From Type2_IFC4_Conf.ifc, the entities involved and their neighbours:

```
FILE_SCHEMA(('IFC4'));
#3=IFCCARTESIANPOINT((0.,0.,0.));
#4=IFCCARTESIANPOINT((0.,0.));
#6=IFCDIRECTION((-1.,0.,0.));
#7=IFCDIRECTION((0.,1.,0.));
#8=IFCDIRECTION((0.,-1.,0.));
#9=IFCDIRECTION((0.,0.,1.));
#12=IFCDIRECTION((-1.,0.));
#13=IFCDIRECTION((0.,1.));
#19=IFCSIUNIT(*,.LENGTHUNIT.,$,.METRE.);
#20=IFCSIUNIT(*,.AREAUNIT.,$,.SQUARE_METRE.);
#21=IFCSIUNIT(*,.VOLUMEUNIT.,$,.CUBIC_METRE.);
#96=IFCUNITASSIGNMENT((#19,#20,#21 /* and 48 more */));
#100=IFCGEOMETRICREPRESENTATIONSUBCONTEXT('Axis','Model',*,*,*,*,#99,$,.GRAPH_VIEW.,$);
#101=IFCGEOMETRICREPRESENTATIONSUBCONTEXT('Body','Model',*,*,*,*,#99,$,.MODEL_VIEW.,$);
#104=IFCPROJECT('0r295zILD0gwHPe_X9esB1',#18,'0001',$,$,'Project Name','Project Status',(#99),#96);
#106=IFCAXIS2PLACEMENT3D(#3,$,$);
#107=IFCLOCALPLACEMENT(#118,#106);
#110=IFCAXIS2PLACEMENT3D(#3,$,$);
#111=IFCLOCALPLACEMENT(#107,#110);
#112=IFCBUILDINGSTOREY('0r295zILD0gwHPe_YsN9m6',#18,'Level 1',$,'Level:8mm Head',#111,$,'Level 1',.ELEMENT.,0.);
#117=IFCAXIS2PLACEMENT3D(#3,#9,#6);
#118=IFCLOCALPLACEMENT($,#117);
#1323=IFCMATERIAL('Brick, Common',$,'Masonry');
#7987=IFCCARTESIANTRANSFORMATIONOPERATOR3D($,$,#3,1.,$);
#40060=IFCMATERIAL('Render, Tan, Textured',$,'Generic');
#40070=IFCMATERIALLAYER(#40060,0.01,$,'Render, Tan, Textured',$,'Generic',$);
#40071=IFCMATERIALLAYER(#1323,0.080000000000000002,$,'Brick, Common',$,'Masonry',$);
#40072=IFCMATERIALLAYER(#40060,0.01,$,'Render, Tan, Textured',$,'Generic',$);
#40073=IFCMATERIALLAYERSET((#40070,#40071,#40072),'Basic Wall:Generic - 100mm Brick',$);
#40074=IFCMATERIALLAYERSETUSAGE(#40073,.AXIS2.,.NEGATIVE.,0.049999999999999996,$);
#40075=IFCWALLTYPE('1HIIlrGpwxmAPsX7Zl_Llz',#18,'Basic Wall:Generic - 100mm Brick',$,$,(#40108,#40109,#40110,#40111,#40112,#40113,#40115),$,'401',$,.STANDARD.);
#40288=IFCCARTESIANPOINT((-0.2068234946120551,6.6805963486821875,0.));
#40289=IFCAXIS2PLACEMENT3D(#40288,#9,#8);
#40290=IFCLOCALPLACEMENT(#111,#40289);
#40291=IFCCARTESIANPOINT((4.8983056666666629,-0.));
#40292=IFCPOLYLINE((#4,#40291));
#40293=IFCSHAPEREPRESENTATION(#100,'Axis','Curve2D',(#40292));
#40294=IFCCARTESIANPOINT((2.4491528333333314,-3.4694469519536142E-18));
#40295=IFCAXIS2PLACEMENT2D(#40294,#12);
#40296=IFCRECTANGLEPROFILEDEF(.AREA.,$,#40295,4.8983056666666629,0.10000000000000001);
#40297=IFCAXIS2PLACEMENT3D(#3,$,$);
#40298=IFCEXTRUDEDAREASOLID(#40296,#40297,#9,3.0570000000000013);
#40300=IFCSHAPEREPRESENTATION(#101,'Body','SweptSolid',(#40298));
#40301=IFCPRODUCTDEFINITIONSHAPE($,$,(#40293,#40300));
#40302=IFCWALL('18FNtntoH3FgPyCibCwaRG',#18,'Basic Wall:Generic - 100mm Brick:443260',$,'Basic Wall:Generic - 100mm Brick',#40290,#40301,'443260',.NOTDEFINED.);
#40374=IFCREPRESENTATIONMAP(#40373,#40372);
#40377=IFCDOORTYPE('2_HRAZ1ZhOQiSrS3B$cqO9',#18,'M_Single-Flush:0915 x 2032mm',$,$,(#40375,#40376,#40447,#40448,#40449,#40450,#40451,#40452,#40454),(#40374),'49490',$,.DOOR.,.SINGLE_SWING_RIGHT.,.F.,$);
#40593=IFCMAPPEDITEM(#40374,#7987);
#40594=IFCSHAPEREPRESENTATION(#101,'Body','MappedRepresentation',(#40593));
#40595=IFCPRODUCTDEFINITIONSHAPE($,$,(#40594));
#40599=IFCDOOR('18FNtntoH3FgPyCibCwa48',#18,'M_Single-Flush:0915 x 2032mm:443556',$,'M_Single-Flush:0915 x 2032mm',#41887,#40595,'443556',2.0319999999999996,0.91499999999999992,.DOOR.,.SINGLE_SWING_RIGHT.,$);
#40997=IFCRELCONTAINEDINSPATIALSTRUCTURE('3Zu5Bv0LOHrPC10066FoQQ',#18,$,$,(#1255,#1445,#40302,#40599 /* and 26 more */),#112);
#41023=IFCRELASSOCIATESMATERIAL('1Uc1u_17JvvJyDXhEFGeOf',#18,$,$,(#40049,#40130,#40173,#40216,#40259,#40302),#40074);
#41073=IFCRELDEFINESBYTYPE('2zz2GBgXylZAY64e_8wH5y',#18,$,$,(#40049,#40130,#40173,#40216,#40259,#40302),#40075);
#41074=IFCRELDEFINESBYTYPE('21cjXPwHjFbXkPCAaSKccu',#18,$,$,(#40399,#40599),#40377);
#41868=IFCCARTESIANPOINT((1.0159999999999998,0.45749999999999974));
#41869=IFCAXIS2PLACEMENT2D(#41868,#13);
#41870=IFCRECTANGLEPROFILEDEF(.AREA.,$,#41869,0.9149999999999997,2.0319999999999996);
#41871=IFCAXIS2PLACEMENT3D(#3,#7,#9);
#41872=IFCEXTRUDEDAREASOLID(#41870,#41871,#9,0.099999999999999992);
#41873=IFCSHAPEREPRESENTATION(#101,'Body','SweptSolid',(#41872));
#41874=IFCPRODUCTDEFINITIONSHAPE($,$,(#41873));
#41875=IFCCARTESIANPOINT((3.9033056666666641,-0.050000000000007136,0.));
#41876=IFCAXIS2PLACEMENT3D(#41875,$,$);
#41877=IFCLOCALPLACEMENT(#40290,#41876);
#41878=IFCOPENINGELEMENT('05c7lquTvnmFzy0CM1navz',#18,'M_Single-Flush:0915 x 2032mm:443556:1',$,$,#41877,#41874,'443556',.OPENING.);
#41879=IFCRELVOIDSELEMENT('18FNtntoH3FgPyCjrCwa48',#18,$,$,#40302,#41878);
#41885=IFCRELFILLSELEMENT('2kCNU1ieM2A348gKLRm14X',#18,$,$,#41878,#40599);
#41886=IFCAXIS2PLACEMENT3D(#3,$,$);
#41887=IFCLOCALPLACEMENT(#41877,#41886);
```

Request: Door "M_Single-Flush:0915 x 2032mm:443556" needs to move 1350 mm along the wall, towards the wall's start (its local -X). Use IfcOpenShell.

```python
import ifcopenshell
import ifcopenshell.api.geometry
import ifcopenshell.util.placement

model = ifcopenshell.open("Type2_IFC4_Conf.ifc")

door = model.by_guid("18FNtntoH3FgPyCibCwa48")
opening = door.FillsVoids[0].RelatingOpeningElement
wall = opening.VoidsElements[0].RelatingBuildingElement

wall_matrix = ifcopenshell.util.placement.get_local_placement(wall.ObjectPlacement)
shift = wall_matrix[:3, 0] * -1.35
before = ifcopenshell.util.placement.get_local_placement(door.ObjectPlacement)[:3, 3].copy()

# The door is placed relative to its opening, so it follows when the opening moves.
matrix = ifcopenshell.util.placement.get_local_placement(opening.ObjectPlacement)
matrix[:3, 3] += shift
ifcopenshell.api.geometry.edit_object_placement(
    model, product=opening, matrix=matrix, is_si=False, should_transform_children=True
)

after = ifcopenshell.util.placement.get_local_placement(door.ObjectPlacement)[:3, 3]
print("door moved by", (after - before).round(3) + 0.0)

model.write("Type2_IFC4_Conf_v2.ifc")
```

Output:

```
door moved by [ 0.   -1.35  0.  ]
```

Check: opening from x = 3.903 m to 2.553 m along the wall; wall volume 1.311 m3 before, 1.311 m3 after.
